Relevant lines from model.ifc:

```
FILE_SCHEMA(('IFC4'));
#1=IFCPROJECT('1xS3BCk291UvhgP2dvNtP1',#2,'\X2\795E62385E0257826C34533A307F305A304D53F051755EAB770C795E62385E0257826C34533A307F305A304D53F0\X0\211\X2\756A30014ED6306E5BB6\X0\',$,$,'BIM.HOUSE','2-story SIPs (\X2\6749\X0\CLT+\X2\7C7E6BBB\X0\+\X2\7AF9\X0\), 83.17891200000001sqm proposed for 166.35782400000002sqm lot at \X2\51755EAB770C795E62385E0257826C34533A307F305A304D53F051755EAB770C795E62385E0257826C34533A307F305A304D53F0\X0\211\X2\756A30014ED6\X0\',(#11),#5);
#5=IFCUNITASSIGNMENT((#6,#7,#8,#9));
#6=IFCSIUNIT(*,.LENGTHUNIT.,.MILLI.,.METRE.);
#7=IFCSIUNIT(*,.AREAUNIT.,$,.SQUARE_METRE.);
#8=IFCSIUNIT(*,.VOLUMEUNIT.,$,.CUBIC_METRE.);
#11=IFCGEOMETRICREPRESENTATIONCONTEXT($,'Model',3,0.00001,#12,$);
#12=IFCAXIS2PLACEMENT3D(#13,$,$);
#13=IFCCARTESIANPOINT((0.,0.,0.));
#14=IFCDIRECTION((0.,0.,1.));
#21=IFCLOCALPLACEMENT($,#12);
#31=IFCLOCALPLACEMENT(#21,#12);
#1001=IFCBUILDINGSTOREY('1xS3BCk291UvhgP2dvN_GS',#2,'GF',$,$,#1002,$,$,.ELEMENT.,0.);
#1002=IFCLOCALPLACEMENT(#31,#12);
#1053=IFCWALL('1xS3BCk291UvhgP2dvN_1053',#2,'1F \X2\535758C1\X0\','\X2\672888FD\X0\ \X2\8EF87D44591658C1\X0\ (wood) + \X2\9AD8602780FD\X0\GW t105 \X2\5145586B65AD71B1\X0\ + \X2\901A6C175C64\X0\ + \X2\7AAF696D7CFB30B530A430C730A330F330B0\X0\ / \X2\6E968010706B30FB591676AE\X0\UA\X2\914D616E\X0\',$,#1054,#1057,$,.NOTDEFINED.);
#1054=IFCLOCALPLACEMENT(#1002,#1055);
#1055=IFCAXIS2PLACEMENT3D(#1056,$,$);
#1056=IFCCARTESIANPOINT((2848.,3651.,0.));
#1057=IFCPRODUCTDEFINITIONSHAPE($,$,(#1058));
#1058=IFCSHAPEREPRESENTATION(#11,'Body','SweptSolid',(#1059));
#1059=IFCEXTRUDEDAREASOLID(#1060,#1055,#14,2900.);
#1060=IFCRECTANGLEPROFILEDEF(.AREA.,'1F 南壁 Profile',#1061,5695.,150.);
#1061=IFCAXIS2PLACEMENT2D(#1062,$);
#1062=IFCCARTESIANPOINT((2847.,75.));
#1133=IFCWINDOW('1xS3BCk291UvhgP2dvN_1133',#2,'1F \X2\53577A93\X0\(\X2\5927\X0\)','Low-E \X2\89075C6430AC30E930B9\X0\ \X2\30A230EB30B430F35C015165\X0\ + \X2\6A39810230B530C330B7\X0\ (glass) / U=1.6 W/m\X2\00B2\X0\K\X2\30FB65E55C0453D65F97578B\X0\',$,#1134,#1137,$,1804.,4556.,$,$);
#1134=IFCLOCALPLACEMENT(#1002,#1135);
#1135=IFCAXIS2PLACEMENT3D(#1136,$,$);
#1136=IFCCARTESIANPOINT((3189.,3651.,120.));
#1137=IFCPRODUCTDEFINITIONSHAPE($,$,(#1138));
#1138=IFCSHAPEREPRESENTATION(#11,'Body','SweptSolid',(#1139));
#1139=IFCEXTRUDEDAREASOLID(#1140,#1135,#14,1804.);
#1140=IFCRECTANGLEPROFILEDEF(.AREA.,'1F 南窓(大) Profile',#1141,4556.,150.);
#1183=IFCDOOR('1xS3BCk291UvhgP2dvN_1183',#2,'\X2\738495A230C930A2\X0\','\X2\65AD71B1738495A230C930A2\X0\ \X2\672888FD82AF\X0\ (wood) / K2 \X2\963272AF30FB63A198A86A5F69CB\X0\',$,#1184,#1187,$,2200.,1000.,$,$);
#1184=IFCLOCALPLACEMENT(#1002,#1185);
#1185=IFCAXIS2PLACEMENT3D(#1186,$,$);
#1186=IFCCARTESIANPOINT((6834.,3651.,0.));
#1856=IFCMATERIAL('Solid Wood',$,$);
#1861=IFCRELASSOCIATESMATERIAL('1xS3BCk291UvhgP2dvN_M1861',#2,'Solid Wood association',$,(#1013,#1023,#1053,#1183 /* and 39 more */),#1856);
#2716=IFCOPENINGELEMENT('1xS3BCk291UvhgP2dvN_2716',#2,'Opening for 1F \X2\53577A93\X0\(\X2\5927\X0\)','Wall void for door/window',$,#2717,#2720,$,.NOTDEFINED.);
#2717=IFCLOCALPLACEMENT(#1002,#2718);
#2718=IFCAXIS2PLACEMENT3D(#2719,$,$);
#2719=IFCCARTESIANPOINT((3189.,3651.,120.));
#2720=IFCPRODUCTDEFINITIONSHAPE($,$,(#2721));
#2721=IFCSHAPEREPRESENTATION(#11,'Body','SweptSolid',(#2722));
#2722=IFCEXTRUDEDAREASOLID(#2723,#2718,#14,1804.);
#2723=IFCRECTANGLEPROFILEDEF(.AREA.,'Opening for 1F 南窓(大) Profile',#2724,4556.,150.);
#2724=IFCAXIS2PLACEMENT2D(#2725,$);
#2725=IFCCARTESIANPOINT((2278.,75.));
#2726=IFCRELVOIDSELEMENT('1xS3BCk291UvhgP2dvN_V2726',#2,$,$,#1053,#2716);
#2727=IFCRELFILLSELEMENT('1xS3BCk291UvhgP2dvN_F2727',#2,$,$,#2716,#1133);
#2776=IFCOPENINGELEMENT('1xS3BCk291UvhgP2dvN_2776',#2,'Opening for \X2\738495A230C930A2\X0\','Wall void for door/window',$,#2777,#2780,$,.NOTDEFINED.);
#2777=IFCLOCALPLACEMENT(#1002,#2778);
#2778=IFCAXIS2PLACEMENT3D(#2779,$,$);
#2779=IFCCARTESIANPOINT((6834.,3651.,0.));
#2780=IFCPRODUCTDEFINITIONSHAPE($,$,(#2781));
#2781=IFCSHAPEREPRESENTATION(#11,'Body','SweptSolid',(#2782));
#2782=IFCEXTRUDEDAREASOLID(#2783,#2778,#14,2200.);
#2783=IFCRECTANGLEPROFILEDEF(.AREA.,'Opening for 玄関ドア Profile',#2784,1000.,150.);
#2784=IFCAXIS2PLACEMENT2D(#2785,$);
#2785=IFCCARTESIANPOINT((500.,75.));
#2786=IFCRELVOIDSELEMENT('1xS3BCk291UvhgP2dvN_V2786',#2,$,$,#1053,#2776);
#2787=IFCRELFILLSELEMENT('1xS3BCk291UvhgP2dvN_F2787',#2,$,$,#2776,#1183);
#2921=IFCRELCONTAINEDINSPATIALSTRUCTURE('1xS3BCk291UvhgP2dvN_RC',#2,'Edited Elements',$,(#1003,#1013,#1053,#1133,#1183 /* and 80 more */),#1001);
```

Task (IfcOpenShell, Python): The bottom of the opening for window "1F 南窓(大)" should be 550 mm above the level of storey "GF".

```python
import numpy as np
import ifcopenshell
import ifcopenshell.api.geometry
import ifcopenshell.geom
import ifcopenshell.util.element
import ifcopenshell.util.placement
import ifcopenshell.util.shape
import ifcopenshell.util.unit

model = ifcopenshell.open("model.ifc")
unit_scale = ifcopenshell.util.unit.calculate_unit_scale(model)

window = model.by_guid("1xS3BCk291UvhgP2dvN_1133")
opening = window.FillsVoids[0].RelatingOpeningElement
storey = ifcopenshell.util.element.get_container(window, ifc_class="IfcBuildingStorey")
level = ifcopenshell.util.placement.get_local_placement(storey.ObjectPlacement)[2, 3]

# The opening's origin need not be at the sill, so measure its lowest point.
shape = ifcopenshell.geom.create_shape(ifcopenshell.geom.settings(), opening)
bottom = ifcopenshell.util.shape.get_shape_bottom_elevation(shape, shape.geometry) / unit_scale
dz = level + 0.55 / unit_scale - bottom

shift = np.array([0.0, 0.0, dz])
# The window is not placed relative to its opening, so move both.
for product in (opening, window):
    matrix = ifcopenshell.util.placement.get_local_placement(product.ObjectPlacement)
    matrix[:3, 3] += shift
    ifcopenshell.api.geometry.edit_object_placement(model, product=product, matrix=matrix, is_si=False)

print(f"moved by {dz * unit_scale:+.3f} m")

model.write("model_edited.ifc")
```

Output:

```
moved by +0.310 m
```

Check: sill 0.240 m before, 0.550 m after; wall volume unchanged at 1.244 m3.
